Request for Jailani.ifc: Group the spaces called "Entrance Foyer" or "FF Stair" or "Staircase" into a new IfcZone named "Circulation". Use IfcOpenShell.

First a look at what the model holds.

```python
import ifcopenshell

model = ifcopenshell.open("Jailani.ifc")
print(model.schema)
seen = {}
for space in model.by_type("IfcSpace"):
    seen[space.Name] = seen.get(space.Name, 0) + 1
for name, count in sorted(seen.items(), key=str):
    print(count, "x", name)
print("zones:", [z.Name for z in model.by_type("IfcZone")][:20])
```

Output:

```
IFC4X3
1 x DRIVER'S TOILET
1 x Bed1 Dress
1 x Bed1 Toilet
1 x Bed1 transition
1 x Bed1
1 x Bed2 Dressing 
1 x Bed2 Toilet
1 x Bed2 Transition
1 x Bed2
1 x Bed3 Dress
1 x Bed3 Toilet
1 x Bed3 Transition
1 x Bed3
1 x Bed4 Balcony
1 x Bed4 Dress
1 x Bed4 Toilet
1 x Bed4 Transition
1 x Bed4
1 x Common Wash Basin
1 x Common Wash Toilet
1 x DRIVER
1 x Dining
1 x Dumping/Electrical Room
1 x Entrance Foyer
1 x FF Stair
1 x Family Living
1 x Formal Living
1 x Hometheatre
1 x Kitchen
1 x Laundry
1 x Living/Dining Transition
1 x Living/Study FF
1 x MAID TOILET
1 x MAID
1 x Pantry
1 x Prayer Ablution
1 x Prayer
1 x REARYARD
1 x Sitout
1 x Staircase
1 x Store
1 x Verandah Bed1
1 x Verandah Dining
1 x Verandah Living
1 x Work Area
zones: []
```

```python
import ifcopenshell
import ifcopenshell.api.group
import ifcopenshell.api.root

model = ifcopenshell.open("Jailani.ifc")

names = {"Entrance Foyer", "FF Stair", "Staircase"}
spaces = [s for s in model.by_type("IfcSpace") if s.Name in names]

zone = ifcopenshell.api.root.create_entity(model, ifc_class="IfcZone", name="Circulation")
ifcopenshell.api.group.assign_group(model, products=spaces, group=zone)
print(len(spaces), "spaces in", zone.Name)

model.write("Jailani_edited.ifc")
```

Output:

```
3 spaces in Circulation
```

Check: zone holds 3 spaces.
